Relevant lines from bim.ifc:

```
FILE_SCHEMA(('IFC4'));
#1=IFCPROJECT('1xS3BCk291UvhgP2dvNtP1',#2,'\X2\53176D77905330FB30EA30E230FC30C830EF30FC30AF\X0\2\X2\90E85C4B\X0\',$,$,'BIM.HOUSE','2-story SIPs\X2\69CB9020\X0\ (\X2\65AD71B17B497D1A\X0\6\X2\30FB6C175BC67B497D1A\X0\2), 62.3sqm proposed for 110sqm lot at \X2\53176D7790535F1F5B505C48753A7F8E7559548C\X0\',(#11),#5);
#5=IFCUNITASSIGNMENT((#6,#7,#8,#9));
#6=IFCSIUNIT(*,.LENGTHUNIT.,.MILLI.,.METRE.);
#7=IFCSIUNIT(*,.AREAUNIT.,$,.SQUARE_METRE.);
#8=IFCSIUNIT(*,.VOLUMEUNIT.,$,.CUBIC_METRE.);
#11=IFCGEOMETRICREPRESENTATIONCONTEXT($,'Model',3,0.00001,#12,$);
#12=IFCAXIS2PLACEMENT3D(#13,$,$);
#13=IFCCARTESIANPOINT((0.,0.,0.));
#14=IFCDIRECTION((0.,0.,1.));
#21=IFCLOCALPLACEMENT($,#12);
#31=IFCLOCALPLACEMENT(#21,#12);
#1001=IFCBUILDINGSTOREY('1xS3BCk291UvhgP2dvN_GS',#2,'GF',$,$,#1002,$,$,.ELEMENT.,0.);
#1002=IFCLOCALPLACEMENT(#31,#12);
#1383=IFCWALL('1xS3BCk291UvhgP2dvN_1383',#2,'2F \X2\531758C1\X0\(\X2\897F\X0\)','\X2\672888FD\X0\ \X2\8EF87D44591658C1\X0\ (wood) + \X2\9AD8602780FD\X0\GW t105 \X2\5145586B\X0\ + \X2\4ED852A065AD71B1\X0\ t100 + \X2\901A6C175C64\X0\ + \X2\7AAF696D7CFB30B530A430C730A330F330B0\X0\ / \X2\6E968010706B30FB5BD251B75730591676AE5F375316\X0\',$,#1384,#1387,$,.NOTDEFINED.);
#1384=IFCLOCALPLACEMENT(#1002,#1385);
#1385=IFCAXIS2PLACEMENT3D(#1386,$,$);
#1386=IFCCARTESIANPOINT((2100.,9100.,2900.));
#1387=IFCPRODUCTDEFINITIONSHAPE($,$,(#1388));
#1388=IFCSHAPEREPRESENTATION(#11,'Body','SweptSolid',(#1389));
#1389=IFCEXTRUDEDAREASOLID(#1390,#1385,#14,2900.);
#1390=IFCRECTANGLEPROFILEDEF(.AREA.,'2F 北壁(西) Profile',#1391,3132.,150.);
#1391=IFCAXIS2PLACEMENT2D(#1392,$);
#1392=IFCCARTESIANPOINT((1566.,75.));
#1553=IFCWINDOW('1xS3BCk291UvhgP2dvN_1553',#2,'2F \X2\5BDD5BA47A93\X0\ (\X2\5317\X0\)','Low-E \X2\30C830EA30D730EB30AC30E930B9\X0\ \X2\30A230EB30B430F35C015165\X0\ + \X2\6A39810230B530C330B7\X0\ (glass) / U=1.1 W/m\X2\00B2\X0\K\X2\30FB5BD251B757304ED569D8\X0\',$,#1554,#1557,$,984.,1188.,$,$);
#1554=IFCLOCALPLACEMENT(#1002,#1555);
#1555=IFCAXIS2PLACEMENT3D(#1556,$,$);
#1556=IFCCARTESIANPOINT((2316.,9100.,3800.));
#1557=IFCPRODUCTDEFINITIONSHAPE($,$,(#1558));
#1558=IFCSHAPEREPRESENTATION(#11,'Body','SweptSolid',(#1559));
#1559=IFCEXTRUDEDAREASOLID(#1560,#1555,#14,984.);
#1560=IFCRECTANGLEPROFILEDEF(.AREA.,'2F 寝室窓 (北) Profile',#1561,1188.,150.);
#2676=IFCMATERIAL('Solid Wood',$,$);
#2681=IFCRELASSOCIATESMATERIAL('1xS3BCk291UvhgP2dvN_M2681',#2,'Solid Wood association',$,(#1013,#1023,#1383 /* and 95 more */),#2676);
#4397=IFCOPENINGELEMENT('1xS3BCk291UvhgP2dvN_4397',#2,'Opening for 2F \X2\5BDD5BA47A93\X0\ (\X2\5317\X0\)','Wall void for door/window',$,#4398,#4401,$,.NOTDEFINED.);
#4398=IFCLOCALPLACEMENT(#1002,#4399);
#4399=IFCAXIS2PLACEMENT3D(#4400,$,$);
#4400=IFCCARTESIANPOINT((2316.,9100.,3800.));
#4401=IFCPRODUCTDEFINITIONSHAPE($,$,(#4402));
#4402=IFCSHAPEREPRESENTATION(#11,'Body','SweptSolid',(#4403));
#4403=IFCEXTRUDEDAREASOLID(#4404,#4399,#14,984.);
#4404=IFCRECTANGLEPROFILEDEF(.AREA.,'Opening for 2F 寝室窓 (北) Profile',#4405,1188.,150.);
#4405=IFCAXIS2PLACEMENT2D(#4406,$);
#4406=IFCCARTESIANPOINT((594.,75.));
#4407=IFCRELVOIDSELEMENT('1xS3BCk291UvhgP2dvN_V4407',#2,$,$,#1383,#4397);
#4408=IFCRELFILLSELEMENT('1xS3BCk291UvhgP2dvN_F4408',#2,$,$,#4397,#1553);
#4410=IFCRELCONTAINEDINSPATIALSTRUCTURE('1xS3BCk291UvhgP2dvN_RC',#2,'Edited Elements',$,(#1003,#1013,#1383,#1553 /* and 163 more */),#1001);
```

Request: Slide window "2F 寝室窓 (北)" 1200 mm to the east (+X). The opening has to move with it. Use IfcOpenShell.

```python
import ifcopenshell
import ifcopenshell.api.geometry
import ifcopenshell.util.placement

model = ifcopenshell.open("bim.ifc")

window = model.by_guid("1xS3BCk291UvhgP2dvN_1553")
opening = window.FillsVoids[0].RelatingOpeningElement
wall = opening.VoidsElements[0].RelatingBuildingElement

wall_matrix = ifcopenshell.util.placement.get_local_placement(wall.ObjectPlacement)
shift = wall_matrix[:3, 0] * 1200.0
before = ifcopenshell.util.placement.get_local_placement(window.ObjectPlacement)[:3, 3].copy()

# The window is not placed relative to its opening, so move both.
for product in (opening, window):
    matrix = ifcopenshell.util.placement.get_local_placement(product.ObjectPlacement)
    matrix[:3, 3] += shift
    ifcopenshell.api.geometry.edit_object_placement(model, product=product, matrix=matrix, is_si=False)

after = ifcopenshell.util.placement.get_local_placement(window.ObjectPlacement)[:3, 3]
print("window moved by", (after - before).round(3) + 0.0)

model.write("bim_edited.ifc")
```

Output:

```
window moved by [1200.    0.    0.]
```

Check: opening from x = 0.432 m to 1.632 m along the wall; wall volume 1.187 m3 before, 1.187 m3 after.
